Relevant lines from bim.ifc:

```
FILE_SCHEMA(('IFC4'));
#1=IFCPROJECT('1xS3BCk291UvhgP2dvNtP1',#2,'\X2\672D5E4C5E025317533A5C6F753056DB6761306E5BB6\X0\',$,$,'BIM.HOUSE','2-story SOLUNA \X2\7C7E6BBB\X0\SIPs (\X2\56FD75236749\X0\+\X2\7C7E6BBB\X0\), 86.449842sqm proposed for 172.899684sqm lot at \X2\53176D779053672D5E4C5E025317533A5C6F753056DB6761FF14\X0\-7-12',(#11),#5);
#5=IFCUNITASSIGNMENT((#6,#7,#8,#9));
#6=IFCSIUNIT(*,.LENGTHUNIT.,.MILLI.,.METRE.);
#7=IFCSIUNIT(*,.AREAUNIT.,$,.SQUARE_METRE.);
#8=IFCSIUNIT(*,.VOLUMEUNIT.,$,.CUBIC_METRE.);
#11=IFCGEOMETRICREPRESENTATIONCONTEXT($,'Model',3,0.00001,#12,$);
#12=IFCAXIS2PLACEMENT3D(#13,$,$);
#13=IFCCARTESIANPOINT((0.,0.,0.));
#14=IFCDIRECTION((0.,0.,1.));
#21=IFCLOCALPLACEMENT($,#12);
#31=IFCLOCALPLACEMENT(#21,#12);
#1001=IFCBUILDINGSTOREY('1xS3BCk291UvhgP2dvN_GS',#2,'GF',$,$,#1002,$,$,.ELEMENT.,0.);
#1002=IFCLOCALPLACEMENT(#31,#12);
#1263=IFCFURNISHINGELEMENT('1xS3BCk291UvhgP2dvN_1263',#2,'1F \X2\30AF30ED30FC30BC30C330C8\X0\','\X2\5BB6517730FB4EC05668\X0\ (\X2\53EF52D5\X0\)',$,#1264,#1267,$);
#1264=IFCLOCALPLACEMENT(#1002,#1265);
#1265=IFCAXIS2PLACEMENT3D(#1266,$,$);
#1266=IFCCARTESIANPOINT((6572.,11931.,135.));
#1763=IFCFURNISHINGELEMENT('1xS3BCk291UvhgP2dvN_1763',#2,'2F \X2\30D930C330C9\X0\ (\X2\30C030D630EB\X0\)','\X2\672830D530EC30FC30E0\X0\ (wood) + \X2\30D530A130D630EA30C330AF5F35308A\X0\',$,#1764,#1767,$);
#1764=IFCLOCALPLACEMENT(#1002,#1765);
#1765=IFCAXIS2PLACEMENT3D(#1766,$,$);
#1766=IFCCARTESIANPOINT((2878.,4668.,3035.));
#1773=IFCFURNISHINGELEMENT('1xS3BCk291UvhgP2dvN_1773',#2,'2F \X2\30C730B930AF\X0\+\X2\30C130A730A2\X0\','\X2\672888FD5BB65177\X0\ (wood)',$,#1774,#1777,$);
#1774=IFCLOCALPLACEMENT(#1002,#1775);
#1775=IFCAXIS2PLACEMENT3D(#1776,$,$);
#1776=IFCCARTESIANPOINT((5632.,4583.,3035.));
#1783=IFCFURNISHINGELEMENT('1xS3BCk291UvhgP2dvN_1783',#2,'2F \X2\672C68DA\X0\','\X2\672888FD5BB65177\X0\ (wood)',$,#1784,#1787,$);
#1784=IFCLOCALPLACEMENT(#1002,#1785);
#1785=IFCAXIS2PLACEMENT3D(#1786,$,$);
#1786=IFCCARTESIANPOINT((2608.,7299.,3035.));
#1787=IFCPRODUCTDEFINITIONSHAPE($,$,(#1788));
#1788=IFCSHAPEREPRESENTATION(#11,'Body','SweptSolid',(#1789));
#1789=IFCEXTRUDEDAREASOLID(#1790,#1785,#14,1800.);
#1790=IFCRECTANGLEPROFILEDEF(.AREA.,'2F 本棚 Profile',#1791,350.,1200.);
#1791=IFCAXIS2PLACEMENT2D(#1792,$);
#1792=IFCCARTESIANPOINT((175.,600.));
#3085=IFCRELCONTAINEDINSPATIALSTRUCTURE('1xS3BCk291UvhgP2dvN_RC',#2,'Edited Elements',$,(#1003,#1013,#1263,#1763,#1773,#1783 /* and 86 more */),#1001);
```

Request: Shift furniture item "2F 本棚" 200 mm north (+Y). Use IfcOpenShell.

```python
import ifcopenshell
import ifcopenshell.api.geometry
import ifcopenshell.util.placement
import ifcopenshell.util.unit

model = ifcopenshell.open("bim.ifc")
unit_scale = ifcopenshell.util.unit.calculate_unit_scale(model)

item = model.by_guid("1xS3BCk291UvhgP2dvN_1783")
matrix = ifcopenshell.util.placement.get_local_placement(item.ObjectPlacement)
matrix[1, 3] += 0.2 / unit_scale
ifcopenshell.api.geometry.edit_object_placement(model, product=item, matrix=matrix, is_si=False)

print(ifcopenshell.util.placement.get_local_placement(item.ObjectPlacement).round(3) + 0.0)

model.write("bim_rev.ifc")
```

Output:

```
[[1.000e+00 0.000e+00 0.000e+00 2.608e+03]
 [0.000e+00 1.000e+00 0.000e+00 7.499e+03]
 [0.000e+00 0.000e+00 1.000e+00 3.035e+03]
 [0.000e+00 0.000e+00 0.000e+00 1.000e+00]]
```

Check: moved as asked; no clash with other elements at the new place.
